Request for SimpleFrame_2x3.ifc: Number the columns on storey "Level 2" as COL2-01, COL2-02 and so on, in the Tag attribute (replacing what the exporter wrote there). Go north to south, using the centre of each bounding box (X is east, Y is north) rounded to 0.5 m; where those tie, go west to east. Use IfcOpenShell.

First a look at what the model holds.

```python
import ifcopenshell
import ifcopenshell.util.element
import ifcopenshell.util.placement

model = ifcopenshell.open("SimpleFrame_2x3.ifc")
print(model.schema)
storey = next(s for s in model.by_type("IfcBuildingStorey") if s.Name == "Level 2")
columns = [e for e in ifcopenshell.util.element.get_decomposition(storey) if e.is_a("IfcColumn")]
for e in sorted(columns, key=lambda e: e.id()):
    origin = ifcopenshell.util.placement.get_local_placement(e.ObjectPlacement)[:3, 3]
    print(e.id(), e.Tag, e.Name, origin.round(2) + 0.0, sep=" | ")
```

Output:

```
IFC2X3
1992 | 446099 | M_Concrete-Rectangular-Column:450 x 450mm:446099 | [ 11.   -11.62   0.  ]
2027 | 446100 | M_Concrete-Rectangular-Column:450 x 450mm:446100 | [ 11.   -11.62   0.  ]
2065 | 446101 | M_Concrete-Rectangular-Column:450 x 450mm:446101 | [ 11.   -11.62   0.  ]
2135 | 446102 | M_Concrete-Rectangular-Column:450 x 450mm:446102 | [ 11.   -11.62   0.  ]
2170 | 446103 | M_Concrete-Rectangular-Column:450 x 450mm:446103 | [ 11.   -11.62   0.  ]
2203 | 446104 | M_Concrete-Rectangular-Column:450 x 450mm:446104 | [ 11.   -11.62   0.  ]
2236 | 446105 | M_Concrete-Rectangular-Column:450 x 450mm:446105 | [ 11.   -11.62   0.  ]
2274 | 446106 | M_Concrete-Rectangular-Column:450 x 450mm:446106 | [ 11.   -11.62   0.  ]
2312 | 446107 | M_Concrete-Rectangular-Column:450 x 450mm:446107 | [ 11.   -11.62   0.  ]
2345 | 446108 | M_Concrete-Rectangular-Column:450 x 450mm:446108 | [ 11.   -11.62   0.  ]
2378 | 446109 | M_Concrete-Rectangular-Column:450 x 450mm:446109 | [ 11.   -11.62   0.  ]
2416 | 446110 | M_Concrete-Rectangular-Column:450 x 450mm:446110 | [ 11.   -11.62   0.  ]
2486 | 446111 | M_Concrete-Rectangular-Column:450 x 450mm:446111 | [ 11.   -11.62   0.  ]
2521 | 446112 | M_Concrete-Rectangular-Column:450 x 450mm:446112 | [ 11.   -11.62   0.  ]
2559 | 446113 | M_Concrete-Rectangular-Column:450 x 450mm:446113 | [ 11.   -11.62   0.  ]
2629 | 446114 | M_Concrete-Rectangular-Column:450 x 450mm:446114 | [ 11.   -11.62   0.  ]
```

```python
import ifcopenshell
import ifcopenshell.geom
import ifcopenshell.util.element
import ifcopenshell.util.shape

model = ifcopenshell.open("SimpleFrame_2x3.ifc")
settings = ifcopenshell.geom.settings()
settings.set("use-world-coords", True)


def centre(element):
    shape = ifcopenshell.geom.create_shape(settings, element)
    return ifcopenshell.util.shape.get_bbox_centroid(shape.geometry)


storey = next(s for s in model.by_type("IfcBuildingStorey") if s.Name == "Level 2")
columns = [e for e in ifcopenshell.util.element.get_decomposition(storey) if e.is_a("IfcColumn")]

# Insertion points can sit at a corner or the storey origin, so sort by the geometry (in metres).
centres = {e: centre(e) for e in columns}
columns.sort(key=lambda e: (-round(centres[e][1] / 0.5), centres[e][0]))

for i, e in enumerate(columns, start=1):
    number = f"COL2-{i:02d}"
    e.Tag = number
    print(e.id(), number)

model.write("SimpleFrame_2x3_edited.ifc")
```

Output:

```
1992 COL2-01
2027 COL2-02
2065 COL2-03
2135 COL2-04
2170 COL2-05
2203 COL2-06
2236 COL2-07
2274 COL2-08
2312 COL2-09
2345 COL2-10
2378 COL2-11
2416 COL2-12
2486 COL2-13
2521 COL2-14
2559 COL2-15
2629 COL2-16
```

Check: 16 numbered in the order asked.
